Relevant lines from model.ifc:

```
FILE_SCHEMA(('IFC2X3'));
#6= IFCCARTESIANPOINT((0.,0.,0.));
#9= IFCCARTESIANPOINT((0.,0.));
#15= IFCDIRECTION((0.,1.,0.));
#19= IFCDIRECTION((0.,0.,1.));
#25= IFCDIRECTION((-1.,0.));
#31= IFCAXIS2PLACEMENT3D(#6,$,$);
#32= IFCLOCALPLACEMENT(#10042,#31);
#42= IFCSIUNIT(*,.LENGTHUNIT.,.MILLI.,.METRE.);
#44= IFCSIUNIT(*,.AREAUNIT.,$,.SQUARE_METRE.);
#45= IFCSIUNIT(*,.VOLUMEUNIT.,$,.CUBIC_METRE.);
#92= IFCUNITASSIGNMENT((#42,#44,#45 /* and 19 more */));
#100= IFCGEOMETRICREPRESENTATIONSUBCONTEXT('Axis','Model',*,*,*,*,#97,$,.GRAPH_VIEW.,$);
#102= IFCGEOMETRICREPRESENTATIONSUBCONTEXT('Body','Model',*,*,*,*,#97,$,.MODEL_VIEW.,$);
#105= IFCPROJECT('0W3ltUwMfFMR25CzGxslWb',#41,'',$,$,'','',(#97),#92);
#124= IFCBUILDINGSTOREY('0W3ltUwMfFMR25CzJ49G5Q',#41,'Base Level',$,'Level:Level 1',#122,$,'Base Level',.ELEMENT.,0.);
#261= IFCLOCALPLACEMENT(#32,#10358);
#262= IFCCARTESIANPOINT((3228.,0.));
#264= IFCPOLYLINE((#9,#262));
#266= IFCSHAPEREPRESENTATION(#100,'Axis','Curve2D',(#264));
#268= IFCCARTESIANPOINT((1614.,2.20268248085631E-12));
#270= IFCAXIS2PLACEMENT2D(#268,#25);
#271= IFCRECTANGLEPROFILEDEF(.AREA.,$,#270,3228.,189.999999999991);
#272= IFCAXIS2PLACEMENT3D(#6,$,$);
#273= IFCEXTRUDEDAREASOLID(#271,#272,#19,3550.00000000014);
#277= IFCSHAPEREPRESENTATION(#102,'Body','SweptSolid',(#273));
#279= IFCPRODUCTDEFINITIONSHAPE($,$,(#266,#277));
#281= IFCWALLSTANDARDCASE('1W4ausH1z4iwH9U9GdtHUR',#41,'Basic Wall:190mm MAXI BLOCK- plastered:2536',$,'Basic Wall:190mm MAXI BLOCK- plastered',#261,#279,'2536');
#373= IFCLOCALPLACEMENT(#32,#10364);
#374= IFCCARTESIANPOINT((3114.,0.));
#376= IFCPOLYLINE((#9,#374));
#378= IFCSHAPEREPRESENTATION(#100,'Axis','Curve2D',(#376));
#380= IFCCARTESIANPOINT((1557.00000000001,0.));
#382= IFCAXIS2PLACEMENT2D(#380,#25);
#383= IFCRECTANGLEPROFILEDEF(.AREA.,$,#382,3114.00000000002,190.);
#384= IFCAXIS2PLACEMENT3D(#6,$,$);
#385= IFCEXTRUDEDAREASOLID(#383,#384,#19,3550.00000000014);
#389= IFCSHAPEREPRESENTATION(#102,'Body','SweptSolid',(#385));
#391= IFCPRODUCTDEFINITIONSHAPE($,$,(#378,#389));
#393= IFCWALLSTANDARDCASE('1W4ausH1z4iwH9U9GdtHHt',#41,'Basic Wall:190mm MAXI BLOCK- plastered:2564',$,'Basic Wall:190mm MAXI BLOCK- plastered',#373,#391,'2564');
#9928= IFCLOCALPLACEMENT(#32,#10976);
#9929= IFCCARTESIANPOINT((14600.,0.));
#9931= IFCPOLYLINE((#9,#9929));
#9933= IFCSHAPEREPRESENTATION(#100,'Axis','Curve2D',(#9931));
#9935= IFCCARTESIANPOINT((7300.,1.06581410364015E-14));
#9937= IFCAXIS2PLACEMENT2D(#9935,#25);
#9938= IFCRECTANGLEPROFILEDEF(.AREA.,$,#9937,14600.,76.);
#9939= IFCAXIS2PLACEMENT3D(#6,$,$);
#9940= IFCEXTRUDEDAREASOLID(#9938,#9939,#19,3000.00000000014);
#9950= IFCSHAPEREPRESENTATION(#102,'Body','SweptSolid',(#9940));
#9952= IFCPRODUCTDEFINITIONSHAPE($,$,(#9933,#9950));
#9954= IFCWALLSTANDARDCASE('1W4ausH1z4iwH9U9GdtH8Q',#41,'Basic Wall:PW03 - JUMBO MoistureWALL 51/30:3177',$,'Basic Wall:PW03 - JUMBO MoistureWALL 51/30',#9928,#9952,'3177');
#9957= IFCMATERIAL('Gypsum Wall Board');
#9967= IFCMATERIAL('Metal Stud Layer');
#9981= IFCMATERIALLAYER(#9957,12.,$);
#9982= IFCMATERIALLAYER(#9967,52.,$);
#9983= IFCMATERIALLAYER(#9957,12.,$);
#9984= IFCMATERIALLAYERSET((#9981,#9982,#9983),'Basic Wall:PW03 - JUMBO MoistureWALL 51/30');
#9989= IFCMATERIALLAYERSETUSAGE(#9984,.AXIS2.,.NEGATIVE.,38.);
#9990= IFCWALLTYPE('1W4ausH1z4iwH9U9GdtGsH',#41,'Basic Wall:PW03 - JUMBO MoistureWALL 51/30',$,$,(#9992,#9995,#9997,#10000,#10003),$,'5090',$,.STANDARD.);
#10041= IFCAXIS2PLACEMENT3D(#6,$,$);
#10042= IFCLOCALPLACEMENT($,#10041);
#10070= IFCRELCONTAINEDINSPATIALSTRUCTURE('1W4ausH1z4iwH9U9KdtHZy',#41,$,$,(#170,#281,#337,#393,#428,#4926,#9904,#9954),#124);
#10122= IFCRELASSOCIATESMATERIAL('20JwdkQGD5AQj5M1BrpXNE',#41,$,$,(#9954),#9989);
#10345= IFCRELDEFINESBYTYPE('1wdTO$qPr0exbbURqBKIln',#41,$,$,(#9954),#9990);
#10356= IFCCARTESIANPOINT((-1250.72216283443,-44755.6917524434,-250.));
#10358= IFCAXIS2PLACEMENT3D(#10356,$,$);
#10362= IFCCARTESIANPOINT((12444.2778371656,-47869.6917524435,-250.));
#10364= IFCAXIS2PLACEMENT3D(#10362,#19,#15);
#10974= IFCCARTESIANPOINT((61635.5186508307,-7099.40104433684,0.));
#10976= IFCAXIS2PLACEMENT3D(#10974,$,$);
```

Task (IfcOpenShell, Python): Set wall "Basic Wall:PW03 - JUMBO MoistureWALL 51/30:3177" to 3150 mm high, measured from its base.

```python
import ifcopenshell
import ifcopenshell.geom
import ifcopenshell.util.representation
import ifcopenshell.util.shape

model = ifcopenshell.open("model.ifc")
settings = ifcopenshell.geom.settings()


def volume(element):
    """Net volume in cubic metres, openings subtracted."""
    shape = ifcopenshell.geom.create_shape(settings, element)
    return ifcopenshell.util.shape.get_volume(shape.geometry)


wall = model.by_guid("1W4ausH1z4iwH9U9GdtH8Q")
before = volume(wall)

body = ifcopenshell.util.representation.get_representation(wall, "Model", "Body")
solid = body.Items[0]
old_height = solid.Depth
solid.Depth = 3150.0
after = volume(wall)

print(f"height {old_height:g} -> {solid.Depth:g}, volume {before:.3f} -> {after:.3f} m3")

model.write("model_edited.ifc")
```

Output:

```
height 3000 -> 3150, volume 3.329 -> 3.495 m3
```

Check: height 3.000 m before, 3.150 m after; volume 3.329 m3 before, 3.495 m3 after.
